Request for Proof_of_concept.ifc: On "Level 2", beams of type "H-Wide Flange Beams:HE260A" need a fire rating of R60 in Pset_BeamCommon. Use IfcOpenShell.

First a look at what the model holds.

```python
import ifcopenshell
import ifcopenshell.util.element

model = ifcopenshell.open("Proof_of_concept.ifc")
print(model.schema)
storey = next(s for s in model.by_type("IfcBuildingStorey") if s.Name == "Level 2")
beams = [e for e in ifcopenshell.util.element.get_decomposition(storey) if e.is_a("IfcBeam")]
seen = {}
for e in beams:
    element_type = ifcopenshell.util.element.get_type(e)
    key = (element_type.Name if element_type != e and element_type else None, ifcopenshell.util.element.get_pset(e, "Pset_BeamCommon", "FireRating"))
    seen[key] = seen.get(key, 0) + 1
for (name, value), count in sorted(seen.items(), key=str):
    print(count, "x", name, "|", value)
```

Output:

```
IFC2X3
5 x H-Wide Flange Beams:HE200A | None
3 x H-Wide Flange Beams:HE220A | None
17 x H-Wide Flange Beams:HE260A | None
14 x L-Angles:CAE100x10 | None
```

```python
import ifcopenshell
import ifcopenshell.api.pset
import ifcopenshell.util.element

model = ifcopenshell.open("Proof_of_concept.ifc")

storey = next(s for s in model.by_type("IfcBuildingStorey") if s.Name == "Level 2")
beams = [e for e in ifcopenshell.util.element.get_decomposition(storey) if e.is_a("IfcBeam")]

count = 0
for e in beams:
    element_type = ifcopenshell.util.element.get_type(e)
    if element_type in (None, e) or element_type.Name != "H-Wide Flange Beams:HE260A":
        continue
    # add_pset returns the element's existing set when there is one.
    pset = ifcopenshell.api.pset.add_pset(model, product=e, name="Pset_BeamCommon")
    ifcopenshell.api.pset.edit_pset(model, pset=pset, properties={"FireRating": "R60"})
    count += 1

print(count, "beams updated")

model.write("Proof_of_concept_updated.ifc")
```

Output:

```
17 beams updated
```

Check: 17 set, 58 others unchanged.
